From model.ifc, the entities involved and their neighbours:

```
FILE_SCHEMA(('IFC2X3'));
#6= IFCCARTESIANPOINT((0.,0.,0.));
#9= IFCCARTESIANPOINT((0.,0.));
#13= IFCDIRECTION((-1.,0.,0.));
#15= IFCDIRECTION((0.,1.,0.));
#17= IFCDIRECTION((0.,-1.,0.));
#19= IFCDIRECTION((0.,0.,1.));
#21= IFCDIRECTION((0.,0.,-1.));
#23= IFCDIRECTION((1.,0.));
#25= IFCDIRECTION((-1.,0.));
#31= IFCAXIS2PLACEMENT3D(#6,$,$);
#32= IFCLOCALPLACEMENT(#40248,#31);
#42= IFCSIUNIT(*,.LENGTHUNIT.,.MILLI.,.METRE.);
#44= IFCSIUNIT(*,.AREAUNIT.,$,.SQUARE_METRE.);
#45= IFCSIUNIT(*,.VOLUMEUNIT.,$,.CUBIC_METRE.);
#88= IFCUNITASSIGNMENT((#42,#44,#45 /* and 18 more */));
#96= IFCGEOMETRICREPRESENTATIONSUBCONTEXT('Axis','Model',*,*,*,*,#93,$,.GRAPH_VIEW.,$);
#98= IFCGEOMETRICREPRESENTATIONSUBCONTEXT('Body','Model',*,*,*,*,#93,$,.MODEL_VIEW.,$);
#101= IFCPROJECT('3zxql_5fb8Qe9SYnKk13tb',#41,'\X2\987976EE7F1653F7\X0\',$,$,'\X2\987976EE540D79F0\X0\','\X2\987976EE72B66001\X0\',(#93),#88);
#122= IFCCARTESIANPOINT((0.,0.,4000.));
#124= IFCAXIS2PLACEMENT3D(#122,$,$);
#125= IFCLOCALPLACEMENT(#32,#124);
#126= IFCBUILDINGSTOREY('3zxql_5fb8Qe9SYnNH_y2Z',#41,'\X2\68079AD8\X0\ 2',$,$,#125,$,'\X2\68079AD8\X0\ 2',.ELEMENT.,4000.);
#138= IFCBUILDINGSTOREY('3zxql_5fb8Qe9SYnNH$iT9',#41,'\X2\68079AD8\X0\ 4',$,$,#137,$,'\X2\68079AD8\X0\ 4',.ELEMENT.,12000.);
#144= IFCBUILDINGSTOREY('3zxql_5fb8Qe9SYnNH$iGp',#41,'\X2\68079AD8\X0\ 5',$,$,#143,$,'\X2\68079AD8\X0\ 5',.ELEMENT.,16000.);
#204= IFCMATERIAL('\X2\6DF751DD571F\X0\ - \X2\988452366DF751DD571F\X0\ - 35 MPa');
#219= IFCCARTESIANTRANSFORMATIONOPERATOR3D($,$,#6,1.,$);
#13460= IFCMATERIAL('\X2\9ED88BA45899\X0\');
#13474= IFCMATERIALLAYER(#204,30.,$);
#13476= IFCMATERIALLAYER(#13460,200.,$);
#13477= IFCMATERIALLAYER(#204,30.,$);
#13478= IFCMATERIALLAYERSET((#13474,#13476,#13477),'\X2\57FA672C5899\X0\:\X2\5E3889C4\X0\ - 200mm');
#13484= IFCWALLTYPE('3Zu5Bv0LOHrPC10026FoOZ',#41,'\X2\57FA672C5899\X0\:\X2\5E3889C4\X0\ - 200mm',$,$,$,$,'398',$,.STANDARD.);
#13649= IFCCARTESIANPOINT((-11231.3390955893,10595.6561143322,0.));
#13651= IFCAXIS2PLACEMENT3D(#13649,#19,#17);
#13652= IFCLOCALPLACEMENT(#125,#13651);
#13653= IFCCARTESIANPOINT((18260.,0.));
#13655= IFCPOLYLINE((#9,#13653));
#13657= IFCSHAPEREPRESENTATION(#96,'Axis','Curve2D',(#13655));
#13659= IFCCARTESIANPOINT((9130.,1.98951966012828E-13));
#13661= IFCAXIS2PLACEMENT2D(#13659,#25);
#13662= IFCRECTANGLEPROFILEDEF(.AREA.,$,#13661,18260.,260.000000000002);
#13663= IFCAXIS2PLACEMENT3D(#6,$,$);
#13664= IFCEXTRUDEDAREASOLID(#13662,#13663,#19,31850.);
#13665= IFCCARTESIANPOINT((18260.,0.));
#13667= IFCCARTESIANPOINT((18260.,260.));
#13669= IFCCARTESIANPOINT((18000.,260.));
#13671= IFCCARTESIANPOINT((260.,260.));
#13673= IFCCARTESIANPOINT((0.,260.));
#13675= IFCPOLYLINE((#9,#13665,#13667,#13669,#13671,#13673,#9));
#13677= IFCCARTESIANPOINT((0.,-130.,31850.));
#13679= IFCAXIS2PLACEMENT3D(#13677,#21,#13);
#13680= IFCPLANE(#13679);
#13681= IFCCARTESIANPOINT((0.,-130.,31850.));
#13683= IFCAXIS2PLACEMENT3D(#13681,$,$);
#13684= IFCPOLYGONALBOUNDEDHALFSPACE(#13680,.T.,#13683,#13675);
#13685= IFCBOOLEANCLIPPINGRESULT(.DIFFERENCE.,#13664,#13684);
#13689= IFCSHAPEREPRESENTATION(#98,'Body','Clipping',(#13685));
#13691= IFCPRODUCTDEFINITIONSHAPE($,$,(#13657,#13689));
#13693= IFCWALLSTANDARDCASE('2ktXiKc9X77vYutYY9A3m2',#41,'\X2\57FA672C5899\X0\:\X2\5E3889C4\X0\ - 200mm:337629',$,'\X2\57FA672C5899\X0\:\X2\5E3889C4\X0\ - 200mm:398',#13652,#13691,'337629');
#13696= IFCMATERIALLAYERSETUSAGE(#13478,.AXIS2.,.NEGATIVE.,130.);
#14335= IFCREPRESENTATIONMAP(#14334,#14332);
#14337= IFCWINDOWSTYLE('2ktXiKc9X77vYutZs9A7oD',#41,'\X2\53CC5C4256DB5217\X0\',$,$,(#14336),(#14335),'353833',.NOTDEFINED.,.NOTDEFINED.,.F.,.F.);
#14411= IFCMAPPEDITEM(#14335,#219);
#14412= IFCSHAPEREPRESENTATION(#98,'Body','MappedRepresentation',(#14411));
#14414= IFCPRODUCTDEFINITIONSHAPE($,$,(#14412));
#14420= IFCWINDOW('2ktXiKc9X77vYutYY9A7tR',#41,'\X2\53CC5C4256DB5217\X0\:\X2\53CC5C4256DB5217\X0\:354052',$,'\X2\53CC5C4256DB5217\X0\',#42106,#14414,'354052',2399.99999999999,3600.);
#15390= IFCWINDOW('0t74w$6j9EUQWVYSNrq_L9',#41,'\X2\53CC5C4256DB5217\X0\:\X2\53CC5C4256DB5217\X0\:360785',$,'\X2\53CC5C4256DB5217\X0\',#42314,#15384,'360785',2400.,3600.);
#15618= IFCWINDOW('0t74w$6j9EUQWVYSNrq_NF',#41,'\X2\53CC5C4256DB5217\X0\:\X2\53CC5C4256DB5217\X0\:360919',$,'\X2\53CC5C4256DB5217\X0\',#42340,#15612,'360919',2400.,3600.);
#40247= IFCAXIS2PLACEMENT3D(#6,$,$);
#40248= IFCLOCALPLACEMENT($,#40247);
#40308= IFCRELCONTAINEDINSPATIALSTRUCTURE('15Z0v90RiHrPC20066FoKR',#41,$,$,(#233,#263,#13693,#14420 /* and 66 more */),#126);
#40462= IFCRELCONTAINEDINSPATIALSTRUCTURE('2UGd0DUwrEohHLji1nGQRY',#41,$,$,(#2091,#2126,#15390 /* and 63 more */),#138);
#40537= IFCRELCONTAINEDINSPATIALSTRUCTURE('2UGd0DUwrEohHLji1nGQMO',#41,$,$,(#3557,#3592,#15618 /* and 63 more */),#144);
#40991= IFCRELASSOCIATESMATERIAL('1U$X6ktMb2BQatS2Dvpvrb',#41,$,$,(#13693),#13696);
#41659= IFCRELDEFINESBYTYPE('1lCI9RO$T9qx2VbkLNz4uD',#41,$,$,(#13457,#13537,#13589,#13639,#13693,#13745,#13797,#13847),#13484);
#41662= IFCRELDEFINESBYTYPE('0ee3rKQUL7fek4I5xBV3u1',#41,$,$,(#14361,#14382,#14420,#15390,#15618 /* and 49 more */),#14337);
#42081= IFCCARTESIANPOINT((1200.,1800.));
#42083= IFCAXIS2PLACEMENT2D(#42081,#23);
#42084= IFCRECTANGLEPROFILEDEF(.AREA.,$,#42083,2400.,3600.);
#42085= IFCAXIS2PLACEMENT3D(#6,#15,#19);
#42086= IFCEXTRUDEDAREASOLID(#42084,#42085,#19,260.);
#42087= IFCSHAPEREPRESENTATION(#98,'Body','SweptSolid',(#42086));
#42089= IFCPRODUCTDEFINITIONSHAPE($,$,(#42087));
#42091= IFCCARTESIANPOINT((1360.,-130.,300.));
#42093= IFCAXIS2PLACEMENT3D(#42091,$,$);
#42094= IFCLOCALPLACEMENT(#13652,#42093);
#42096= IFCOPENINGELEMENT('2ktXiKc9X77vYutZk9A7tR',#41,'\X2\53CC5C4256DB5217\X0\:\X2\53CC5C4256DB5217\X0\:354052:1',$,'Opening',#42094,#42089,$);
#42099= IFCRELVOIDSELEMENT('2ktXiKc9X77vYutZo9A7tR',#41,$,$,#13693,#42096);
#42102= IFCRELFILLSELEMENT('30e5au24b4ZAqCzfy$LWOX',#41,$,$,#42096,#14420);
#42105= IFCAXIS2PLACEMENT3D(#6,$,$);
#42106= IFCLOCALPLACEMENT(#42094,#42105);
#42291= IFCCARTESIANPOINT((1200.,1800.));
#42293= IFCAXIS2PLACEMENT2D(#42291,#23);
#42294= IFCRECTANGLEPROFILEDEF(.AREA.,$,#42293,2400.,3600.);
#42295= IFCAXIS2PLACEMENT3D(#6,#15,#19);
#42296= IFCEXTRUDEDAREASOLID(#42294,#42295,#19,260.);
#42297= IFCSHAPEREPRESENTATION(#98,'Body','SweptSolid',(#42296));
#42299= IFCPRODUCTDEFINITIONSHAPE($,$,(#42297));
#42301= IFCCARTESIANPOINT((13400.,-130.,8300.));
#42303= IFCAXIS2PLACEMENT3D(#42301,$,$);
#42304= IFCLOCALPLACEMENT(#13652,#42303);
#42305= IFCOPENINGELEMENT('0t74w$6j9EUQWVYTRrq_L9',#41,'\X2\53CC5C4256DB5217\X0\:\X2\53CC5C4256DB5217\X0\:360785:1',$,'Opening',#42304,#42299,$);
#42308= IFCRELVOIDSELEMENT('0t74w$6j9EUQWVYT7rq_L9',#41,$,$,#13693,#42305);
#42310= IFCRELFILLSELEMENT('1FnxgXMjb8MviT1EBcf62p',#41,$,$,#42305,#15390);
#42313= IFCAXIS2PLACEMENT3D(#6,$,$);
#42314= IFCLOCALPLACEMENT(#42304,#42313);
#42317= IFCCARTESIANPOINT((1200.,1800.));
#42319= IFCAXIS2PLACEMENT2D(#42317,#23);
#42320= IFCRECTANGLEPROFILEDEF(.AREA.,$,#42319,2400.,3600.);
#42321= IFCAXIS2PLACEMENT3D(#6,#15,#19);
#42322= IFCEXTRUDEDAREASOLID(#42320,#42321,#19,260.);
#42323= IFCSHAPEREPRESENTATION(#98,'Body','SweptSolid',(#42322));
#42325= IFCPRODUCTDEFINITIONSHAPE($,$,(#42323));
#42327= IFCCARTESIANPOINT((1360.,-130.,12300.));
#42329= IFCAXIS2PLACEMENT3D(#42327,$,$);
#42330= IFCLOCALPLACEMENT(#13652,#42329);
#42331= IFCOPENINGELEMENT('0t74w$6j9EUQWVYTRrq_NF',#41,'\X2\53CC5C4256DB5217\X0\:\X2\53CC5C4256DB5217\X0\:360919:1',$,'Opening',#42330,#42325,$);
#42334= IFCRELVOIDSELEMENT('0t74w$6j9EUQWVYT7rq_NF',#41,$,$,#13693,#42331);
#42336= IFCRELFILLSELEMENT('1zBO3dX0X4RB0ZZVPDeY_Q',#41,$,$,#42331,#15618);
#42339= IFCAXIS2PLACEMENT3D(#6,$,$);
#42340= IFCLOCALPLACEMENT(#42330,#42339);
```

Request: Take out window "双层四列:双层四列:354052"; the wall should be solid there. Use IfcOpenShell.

```python
import ifcopenshell
import ifcopenshell.api.feature
import ifcopenshell.api.root
import ifcopenshell.geom
import ifcopenshell.util.shape

model = ifcopenshell.open("model.ifc")
settings = ifcopenshell.geom.settings()


def volume(element):
    """Net volume in cubic metres, openings subtracted."""
    shape = ifcopenshell.geom.create_shape(settings, element)
    return ifcopenshell.util.shape.get_volume(shape.geometry)


window = model.by_guid("2ktXiKc9X77vYutYY9A7tR")
opening = window.FillsVoids[0].RelatingOpeningElement
wall = opening.VoidsElements[0].RelatingBuildingElement
before = volume(wall)

ifcopenshell.api.root.remove_product(model, product=window)
ifcopenshell.api.feature.remove_feature(model, feature=opening)

after = volume(wall)

print(f"wall volume {before:.3f} -> {after:.3f} m3")

model.write("model_rev.ifc")
```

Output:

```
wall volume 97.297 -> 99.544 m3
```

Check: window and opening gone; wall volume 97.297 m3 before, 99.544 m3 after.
